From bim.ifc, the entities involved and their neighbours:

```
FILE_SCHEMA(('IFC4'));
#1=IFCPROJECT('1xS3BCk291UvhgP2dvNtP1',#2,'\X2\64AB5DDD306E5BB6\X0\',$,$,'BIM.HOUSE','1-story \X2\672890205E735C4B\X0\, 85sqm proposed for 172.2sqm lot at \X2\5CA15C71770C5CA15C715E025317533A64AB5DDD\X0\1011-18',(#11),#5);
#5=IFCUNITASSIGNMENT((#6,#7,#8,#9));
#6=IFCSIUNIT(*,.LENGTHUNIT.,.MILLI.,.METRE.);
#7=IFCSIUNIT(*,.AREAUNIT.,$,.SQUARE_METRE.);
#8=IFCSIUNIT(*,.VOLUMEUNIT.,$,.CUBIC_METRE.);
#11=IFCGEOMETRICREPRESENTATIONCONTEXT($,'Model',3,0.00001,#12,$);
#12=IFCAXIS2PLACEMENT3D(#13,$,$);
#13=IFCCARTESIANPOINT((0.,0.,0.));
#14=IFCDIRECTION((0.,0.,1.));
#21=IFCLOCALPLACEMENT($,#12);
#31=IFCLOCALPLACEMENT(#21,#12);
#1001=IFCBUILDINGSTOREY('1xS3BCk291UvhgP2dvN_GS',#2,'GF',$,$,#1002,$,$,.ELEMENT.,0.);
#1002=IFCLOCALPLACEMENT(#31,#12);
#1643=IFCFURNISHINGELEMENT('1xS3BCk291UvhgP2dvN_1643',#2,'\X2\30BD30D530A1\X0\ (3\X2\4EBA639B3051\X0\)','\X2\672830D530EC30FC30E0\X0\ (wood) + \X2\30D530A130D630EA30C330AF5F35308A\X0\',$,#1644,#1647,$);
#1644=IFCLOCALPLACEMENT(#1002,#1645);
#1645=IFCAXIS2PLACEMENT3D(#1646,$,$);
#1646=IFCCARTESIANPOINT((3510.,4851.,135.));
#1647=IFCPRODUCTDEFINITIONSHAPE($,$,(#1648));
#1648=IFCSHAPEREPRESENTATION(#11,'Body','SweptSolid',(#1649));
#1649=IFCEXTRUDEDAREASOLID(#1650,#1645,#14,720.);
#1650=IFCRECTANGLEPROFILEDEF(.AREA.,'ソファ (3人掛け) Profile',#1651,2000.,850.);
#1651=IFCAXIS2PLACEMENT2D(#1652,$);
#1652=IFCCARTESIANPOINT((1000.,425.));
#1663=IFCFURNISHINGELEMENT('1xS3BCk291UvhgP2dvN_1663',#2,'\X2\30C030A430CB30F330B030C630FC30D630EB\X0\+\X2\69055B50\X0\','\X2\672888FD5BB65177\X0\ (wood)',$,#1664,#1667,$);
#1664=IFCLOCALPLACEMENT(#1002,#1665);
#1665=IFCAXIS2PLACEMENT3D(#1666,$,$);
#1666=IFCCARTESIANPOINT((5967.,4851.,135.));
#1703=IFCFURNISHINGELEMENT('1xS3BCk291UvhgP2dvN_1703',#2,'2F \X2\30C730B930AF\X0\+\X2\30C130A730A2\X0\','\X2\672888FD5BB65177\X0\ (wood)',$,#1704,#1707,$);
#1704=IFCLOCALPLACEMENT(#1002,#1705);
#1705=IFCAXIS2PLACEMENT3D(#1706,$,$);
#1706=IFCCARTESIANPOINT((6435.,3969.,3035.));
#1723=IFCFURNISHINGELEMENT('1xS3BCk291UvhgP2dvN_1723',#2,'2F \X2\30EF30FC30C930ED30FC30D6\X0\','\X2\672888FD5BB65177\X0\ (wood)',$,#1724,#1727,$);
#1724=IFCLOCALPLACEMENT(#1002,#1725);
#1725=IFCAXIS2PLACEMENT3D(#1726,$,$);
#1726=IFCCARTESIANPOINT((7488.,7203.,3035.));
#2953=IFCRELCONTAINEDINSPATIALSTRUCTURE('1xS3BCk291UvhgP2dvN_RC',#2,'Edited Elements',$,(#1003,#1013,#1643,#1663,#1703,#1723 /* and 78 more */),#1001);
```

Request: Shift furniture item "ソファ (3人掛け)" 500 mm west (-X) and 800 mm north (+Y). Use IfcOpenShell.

```python
import ifcopenshell
import ifcopenshell.api.geometry
import ifcopenshell.util.placement
import ifcopenshell.util.unit

model = ifcopenshell.open("bim.ifc")
unit_scale = ifcopenshell.util.unit.calculate_unit_scale(model)

item = model.by_guid("1xS3BCk291UvhgP2dvN_1643")
matrix = ifcopenshell.util.placement.get_local_placement(item.ObjectPlacement)
matrix[0, 3] -= 0.5 / unit_scale
matrix[1, 3] += 0.8 / unit_scale
ifcopenshell.api.geometry.edit_object_placement(model, product=item, matrix=matrix, is_si=False)

print(ifcopenshell.util.placement.get_local_placement(item.ObjectPlacement).round(3) + 0.0)

model.write("bim_v2.ifc")
```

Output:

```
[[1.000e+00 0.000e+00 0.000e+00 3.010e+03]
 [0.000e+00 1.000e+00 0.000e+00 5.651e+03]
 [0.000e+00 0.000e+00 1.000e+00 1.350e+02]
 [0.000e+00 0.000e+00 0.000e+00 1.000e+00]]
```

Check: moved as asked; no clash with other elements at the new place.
